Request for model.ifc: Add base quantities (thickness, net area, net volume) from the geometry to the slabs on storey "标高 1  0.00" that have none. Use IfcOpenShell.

First a look at what the model holds.

```python
import ifcopenshell
import ifcopenshell.util.element
import ifcopenshell.util.unit

model = ifcopenshell.open("model.ifc")
print(model.schema)
for unit_type in ("LENGTHUNIT", "AREAUNIT", "VOLUMEUNIT"):
    print(unit_type, ifcopenshell.util.unit.calculate_unit_scale(model, unit_type))
storey = next(s for s in model.by_type("IfcBuildingStorey") if s.Name == "标高 1  0.00")
slabs = [e for e in ifcopenshell.util.element.get_decomposition(storey) if e.is_a("IfcSlab")]
for e in sorted(slabs, key=lambda e: e.id()):
    print(e.id(), e.is_a(), e.Name, list(ifcopenshell.util.element.get_psets(e, qtos_only=True)), sep=" | ")
```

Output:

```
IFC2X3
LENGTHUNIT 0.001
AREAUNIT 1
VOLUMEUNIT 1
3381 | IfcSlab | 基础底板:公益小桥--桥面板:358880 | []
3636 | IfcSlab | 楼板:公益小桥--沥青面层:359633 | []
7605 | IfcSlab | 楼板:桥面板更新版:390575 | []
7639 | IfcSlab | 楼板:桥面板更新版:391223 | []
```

```python
import ifcopenshell
import ifcopenshell.api.pset
import ifcopenshell.geom
import ifcopenshell.util.element
import ifcopenshell.util.shape
import ifcopenshell.util.unit

model = ifcopenshell.open("model.ifc")
unit_scale = ifcopenshell.util.unit.calculate_unit_scale(model)
area_scale = ifcopenshell.util.unit.calculate_unit_scale(model, "AREAUNIT")
volume_scale = ifcopenshell.util.unit.calculate_unit_scale(model, "VOLUMEUNIT")
settings = ifcopenshell.geom.settings()

storey = next(s for s in model.by_type("IfcBuildingStorey") if s.Name == "标高 1  0.00")
slabs = [e for e in ifcopenshell.util.element.get_decomposition(storey) if e.is_a("IfcSlab")]

for e in sorted(slabs, key=lambda e: e.id()):
    if ifcopenshell.util.element.get_psets(e, qtos_only=True, should_inherit=False):
        continue
    # Geometry comes back in metres, in the element's own axes.
    shape = ifcopenshell.geom.create_shape(settings, e)
    values = {
        "Width": ifcopenshell.util.shape.get_z(shape.geometry) / unit_scale,
        "NetArea": ifcopenshell.util.shape.get_footprint_area(shape.geometry) / area_scale,
        "NetVolume": ifcopenshell.util.shape.get_volume(shape.geometry) / volume_scale,
    }
    qto = ifcopenshell.api.pset.add_qto(model, product=e, name="BaseQuantities")
    ifcopenshell.api.pset.edit_qto(model, qto=qto, properties=values)
    print(e.id(), {k: round(v, 3) for k, v in values.items()})

model.write("model_rev.ifc")
```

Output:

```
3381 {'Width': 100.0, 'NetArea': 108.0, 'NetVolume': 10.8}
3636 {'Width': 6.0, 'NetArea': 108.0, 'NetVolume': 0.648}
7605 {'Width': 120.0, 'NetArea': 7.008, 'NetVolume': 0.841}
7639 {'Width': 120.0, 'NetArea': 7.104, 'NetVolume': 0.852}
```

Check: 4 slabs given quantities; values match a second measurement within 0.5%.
